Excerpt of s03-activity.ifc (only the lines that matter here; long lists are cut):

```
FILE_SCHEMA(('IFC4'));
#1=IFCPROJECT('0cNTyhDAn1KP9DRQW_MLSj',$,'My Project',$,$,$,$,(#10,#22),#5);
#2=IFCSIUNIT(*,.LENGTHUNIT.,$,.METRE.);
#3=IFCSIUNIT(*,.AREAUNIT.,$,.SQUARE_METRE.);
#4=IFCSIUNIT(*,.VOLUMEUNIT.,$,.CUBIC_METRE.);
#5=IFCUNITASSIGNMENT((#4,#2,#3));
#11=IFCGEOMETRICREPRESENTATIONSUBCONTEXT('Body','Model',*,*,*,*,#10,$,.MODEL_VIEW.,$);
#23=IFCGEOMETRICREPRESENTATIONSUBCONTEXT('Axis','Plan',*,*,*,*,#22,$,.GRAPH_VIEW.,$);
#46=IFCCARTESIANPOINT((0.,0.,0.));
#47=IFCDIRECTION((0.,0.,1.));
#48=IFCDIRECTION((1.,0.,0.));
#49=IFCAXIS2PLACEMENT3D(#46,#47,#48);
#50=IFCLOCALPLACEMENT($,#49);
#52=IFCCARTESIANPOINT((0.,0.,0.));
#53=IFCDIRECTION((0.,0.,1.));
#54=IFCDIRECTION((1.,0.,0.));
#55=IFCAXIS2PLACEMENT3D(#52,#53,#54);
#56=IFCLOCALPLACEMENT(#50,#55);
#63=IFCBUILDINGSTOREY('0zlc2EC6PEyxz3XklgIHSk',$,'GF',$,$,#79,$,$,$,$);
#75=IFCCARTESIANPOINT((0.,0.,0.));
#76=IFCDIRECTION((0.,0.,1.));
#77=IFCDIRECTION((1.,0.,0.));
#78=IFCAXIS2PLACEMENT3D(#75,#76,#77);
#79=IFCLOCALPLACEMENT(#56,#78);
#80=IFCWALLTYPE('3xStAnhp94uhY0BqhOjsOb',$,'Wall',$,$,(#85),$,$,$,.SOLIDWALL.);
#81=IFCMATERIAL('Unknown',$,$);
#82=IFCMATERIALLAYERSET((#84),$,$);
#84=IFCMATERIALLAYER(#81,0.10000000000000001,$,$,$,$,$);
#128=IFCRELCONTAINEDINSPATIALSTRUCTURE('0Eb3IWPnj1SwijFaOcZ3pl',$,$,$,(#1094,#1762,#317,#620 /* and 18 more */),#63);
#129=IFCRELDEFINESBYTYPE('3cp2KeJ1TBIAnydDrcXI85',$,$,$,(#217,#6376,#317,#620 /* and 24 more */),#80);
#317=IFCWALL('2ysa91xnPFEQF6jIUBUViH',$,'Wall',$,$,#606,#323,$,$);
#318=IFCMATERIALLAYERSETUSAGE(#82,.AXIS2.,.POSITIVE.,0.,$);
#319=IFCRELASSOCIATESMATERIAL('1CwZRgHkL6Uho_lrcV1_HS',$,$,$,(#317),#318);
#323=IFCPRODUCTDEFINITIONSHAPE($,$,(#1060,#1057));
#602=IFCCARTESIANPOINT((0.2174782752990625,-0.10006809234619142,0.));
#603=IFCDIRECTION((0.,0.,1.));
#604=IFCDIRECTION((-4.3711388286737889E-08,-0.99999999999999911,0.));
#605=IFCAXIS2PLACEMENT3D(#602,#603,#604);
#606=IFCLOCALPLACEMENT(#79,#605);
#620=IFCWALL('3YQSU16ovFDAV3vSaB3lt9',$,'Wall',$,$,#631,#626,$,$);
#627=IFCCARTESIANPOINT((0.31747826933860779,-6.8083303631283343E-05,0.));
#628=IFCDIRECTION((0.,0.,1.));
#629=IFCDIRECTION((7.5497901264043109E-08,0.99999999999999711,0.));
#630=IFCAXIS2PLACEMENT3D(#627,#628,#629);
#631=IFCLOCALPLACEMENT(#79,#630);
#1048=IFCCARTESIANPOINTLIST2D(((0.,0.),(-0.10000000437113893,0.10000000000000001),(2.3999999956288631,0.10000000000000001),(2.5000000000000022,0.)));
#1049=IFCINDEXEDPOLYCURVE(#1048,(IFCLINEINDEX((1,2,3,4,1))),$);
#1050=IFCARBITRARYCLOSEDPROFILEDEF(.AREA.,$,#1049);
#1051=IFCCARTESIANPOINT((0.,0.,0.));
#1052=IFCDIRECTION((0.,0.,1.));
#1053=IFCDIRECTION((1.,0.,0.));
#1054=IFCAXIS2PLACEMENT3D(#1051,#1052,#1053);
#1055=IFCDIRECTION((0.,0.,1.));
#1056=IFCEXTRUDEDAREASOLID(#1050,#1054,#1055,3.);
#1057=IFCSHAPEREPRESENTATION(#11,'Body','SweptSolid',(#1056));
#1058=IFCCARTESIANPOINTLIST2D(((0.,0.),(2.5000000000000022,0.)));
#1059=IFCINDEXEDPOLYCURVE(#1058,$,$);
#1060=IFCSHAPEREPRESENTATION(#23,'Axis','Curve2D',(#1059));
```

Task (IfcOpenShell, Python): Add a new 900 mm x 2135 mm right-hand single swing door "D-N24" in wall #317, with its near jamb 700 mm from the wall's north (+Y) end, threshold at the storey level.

```python
import numpy as np
import ifcopenshell
import ifcopenshell.api.feature
import ifcopenshell.api.geometry
import ifcopenshell.api.root
import ifcopenshell.api.spatial
import ifcopenshell.geom
import ifcopenshell.util.element
import ifcopenshell.util.placement
import ifcopenshell.util.representation
import ifcopenshell.util.shape
import ifcopenshell.util.unit

model = ifcopenshell.open("s03-activity.ifc")
unit_scale = ifcopenshell.util.unit.calculate_unit_scale(model)
settings = ifcopenshell.geom.settings()


def volume(element):
    """Net volume in cubic metres, openings subtracted."""
    shape = ifcopenshell.geom.create_shape(settings, element)
    return ifcopenshell.util.shape.get_volume(shape.geometry)


wall = model.by_id(317)
storey = ifcopenshell.util.element.get_container(wall, ifc_class="IfcBuildingStorey")
context = ifcopenshell.util.representation.get_context(model, "Model", "Body", "MODEL_VIEW")
before = volume(wall)

width, height, from_end, sill = 0.9, 2.135, 0.7, 0.0  # metres

# The wall runs along its own X axis, and the end named is its -X end.
wall_shape = ifcopenshell.geom.create_shape(settings, wall)
x, y, z = ifcopenshell.util.shape.get_vertices(wall_shape.geometry).T
start = x.min() + from_end
face, thickness = float(y.min()), float(y.max() - y.min())
wall_matrix = ifcopenshell.util.placement.get_local_placement(wall.ObjectPlacement)
level = ifcopenshell.util.placement.get_local_placement(storey.ObjectPlacement)[2, 3]


def in_wall(x, y):
    """Placement at x, y metres in the wall's axes, at sill height."""
    matrix = wall_matrix.copy()
    matrix[:, 3] = wall_matrix @ np.array([x / unit_scale, y / unit_scale, 0.0, 1.0])
    matrix[2, 3] = level + sill / unit_scale
    return matrix


# Opening: a box that overshoots both wall faces by 50 mm.
opening = ifcopenshell.api.root.create_entity(model, ifc_class="IfcOpeningElement", predefined_type="OPENING")
box = ifcopenshell.api.geometry.add_wall_representation(
    model, context=context, length=width, height=height, thickness=thickness + 0.1
)
ifcopenshell.api.geometry.assign_representation(model, product=opening, representation=box)
ifcopenshell.api.geometry.edit_object_placement(model, product=opening, matrix=in_wall(start, face - 0.05), is_si=False)
ifcopenshell.api.feature.add_feature(model, feature=opening, element=wall)

door = ifcopenshell.api.root.create_entity(model, ifc_class="IfcDoor", name="D-N24", predefined_type="DOOR")
door.OverallWidth, door.OverallHeight = width / unit_scale, height / unit_scale
door.OperationType = "SINGLE_SWING_RIGHT"
body = ifcopenshell.api.geometry.add_door_representation(
    model,
    context=context,
    overall_width=door.OverallWidth,
    overall_height=door.OverallHeight,
    operation_type="SINGLE_SWING_RIGHT",
    lining_properties={"LiningDepth": thickness / unit_scale, "ThresholdDepth": thickness / unit_scale},
)
ifcopenshell.api.geometry.assign_representation(model, product=door, representation=body)
ifcopenshell.api.spatial.assign_container(model, products=[door], relating_structure=storey)
ifcopenshell.api.feature.add_filling(model, opening=opening, element=door)

# The lining spans the wall, so the door starts at the wall face.
ifcopenshell.api.geometry.edit_object_placement(model, product=door, matrix=in_wall(start, face), is_si=False)

after = volume(wall)

print(f"wall volume {before:.3f} -> {after:.3f} m3")

model.write("s03-activity-out.ifc")
```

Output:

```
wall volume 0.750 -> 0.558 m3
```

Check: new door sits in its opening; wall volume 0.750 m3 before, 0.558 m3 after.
